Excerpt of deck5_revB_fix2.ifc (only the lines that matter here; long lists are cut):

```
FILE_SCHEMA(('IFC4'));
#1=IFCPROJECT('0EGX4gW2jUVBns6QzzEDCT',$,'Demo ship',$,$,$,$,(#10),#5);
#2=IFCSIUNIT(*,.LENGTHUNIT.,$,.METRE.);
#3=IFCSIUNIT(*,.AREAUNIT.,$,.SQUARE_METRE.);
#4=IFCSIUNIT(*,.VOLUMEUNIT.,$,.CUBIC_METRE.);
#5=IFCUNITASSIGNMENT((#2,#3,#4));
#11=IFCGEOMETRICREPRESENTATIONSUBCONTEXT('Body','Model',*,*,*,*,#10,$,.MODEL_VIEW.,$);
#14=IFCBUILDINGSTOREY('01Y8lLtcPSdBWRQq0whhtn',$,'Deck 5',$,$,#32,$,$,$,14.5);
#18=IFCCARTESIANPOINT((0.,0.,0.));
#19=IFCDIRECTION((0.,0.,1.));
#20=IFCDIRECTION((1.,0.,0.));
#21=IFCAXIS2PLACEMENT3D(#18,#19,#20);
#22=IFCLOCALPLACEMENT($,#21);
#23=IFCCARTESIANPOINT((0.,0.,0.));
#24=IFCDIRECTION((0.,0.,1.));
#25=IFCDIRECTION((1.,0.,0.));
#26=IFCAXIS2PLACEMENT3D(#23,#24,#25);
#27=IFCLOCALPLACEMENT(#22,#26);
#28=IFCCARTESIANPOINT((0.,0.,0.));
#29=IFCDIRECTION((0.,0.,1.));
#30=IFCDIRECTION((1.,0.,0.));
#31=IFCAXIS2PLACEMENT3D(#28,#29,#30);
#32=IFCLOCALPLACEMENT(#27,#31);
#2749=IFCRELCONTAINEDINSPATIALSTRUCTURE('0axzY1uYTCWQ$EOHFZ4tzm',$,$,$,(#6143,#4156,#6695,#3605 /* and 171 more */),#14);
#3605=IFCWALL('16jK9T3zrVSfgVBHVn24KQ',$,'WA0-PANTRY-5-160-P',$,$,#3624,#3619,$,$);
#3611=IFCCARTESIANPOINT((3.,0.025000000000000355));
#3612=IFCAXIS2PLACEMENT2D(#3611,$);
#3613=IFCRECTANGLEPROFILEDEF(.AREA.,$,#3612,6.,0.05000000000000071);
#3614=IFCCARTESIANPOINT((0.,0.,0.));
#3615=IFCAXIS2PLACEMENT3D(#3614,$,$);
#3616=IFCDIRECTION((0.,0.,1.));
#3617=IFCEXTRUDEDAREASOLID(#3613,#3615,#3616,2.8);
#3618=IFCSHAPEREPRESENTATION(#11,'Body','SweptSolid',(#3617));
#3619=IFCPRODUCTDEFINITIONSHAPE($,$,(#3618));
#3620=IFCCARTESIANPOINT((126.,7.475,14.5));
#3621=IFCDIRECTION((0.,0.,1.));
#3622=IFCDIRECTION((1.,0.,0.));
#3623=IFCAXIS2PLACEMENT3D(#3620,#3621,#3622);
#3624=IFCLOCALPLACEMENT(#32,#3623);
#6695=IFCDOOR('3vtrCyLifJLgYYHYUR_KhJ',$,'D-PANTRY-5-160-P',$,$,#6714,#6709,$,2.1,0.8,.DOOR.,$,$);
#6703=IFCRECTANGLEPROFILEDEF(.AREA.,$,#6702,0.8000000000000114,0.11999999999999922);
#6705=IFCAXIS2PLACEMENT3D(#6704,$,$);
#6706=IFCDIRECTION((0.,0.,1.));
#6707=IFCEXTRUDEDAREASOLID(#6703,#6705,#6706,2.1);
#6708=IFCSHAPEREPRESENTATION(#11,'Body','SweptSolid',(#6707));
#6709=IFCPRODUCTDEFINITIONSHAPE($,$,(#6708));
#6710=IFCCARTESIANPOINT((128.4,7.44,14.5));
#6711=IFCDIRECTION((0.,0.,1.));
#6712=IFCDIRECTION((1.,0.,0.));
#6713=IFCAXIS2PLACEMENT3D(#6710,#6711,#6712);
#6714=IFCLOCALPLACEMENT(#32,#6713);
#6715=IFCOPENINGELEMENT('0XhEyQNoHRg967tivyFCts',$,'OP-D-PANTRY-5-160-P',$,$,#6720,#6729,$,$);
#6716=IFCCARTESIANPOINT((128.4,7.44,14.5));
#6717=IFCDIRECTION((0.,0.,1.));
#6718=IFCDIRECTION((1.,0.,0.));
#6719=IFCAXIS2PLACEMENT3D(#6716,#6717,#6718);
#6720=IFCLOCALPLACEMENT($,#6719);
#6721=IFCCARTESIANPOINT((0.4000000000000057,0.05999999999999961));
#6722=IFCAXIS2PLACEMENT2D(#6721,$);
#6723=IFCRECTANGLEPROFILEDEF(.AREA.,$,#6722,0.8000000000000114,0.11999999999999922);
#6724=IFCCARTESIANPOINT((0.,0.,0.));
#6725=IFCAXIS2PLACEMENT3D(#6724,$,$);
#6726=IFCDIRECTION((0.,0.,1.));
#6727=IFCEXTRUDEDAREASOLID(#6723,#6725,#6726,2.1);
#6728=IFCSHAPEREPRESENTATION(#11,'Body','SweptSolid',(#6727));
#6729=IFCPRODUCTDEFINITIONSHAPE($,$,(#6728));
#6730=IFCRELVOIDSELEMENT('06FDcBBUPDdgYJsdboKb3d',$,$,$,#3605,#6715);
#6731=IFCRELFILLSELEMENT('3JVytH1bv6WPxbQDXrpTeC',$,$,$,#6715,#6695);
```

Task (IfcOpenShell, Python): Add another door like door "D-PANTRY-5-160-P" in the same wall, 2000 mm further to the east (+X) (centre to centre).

```python
import ifcopenshell
import ifcopenshell.api.feature
import ifcopenshell.api.geometry
import ifcopenshell.api.root
import ifcopenshell.geom
import ifcopenshell.util.element
import ifcopenshell.util.placement
import ifcopenshell.util.shape

model = ifcopenshell.open("deck5_revB_fix2.ifc")
settings = ifcopenshell.geom.settings()


def volume(element):
    """Net volume in cubic metres, openings subtracted."""
    shape = ifcopenshell.geom.create_shape(settings, element)
    return ifcopenshell.util.shape.get_volume(shape.geometry)


door = model.by_id(6695)
opening = door.FillsVoids[0].RelatingOpeningElement
wall = opening.VoidsElements[0].RelatingBuildingElement
before = volume(wall)
shift = ifcopenshell.util.placement.get_local_placement(wall.ObjectPlacement)[:3, 0] * 2.0

# copy_class copies the void relationship, type, container and properties, but no geometry.
new_opening = ifcopenshell.api.root.copy_class(model, product=opening)
new_opening.Representation = ifcopenshell.util.element.copy_deep(
    model, opening.Representation, exclude=["IfcGeometricRepresentationContext", "IfcRepresentationMap"]
)
new_door = ifcopenshell.api.root.copy_class(model, product=door)
new_door.Representation = ifcopenshell.util.element.copy_deep(
    model, door.Representation, exclude=["IfcGeometricRepresentationContext", "IfcRepresentationMap"]
)
ifcopenshell.api.feature.add_filling(model, opening=new_opening, element=new_door)

for old, new in ((opening, new_opening), (door, new_door)):
    matrix = ifcopenshell.util.placement.get_local_placement(old.ObjectPlacement)
    matrix[:3, 3] += shift
    ifcopenshell.api.geometry.edit_object_placement(model, product=new, matrix=matrix, is_si=False)

after = volume(wall)

print(f"wall volume {before:.3f} -> {after:.3f} m3")

model.write("deck5_revB_fix2_edited.ifc")
```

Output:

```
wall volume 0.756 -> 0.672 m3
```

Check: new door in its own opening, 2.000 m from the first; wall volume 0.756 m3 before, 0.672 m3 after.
